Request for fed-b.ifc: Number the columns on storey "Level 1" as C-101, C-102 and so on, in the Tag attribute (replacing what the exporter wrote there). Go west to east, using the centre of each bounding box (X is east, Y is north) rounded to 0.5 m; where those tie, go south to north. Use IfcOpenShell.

First a look at what the model holds.

```python
import ifcopenshell
import ifcopenshell.util.element
import ifcopenshell.util.placement

model = ifcopenshell.open("fed-b.ifc")
print(model.schema)
storey = next(s for s in model.by_type("IfcBuildingStorey") if s.Name == "Level 1")
columns = [e for e in ifcopenshell.util.element.get_decomposition(storey) if e.is_a("IfcColumn")]
for e in sorted(columns, key=lambda e: e.id()):
    origin = ifcopenshell.util.placement.get_local_placement(e.ObjectPlacement)[:3, 3]
    print(e.id(), e.Tag, e.Name, origin.round(2) + 0.0, sep=" | ")
```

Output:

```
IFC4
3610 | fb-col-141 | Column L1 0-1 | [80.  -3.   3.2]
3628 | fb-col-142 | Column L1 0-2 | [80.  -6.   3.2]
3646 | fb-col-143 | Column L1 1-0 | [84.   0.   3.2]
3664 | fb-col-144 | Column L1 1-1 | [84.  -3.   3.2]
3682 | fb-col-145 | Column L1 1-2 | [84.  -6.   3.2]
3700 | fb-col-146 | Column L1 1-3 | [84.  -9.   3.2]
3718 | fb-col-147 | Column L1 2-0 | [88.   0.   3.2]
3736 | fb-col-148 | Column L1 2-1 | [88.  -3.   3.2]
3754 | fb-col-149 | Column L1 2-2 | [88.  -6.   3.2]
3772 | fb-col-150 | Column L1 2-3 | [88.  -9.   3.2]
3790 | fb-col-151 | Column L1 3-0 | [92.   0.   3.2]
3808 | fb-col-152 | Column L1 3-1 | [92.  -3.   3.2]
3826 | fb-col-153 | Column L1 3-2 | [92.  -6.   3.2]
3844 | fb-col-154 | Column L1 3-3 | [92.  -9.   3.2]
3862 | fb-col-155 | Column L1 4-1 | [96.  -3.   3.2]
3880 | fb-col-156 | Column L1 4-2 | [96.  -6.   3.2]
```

```python
import ifcopenshell
import ifcopenshell.geom
import ifcopenshell.util.element
import ifcopenshell.util.shape

model = ifcopenshell.open("fed-b.ifc")
settings = ifcopenshell.geom.settings()
settings.set("use-world-coords", True)


def centre(element):
    shape = ifcopenshell.geom.create_shape(settings, element)
    return ifcopenshell.util.shape.get_bbox_centroid(shape.geometry)


storey = next(s for s in model.by_type("IfcBuildingStorey") if s.Name == "Level 1")
columns = [e for e in ifcopenshell.util.element.get_decomposition(storey) if e.is_a("IfcColumn")]

# Insertion points can sit at a corner or the storey origin, so sort by the geometry (in metres).
centres = {e: centre(e) for e in columns}
columns.sort(key=lambda e: (round(centres[e][0] / 0.5), centres[e][1]))

for i, e in enumerate(columns, start=1):
    number = f"C-1{i:02d}"
    e.Tag = number
    print(e.id(), number)

model.write("fed-b-out.ifc")
```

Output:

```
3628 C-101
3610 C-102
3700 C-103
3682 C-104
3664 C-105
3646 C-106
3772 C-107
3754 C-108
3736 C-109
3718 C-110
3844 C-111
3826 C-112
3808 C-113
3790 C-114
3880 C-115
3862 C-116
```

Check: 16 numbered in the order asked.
